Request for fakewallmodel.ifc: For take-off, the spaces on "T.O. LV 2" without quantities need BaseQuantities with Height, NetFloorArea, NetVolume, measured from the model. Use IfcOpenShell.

First a look at what the model holds.

```python
import ifcopenshell
import ifcopenshell.util.element
import ifcopenshell.util.unit

model = ifcopenshell.open("fakewallmodel.ifc")
print(model.schema)
for unit_type in ("LENGTHUNIT", "AREAUNIT", "VOLUMEUNIT"):
    print(unit_type, ifcopenshell.util.unit.calculate_unit_scale(model, unit_type))
storey = next(s for s in model.by_type("IfcBuildingStorey") if s.Name == "T.O. LV 2")
spaces = [e for e in ifcopenshell.util.element.get_decomposition(storey) if e.is_a("IfcSpace")]
for e in sorted(spaces, key=lambda e: e.id()):
    print(e.id(), e.is_a(), e.Name, list(ifcopenshell.util.element.get_psets(e, qtos_only=True)), sep=" | ")
```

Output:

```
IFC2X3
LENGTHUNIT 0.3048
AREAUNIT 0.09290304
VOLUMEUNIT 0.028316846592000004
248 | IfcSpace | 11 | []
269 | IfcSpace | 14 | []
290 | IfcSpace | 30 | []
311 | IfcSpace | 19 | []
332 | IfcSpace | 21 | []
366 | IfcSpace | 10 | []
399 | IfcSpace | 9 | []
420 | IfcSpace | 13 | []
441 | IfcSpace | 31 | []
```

```python
import ifcopenshell
import ifcopenshell.api.pset
import ifcopenshell.geom
import ifcopenshell.util.element
import ifcopenshell.util.shape
import ifcopenshell.util.unit

model = ifcopenshell.open("fakewallmodel.ifc")
unit_scale = ifcopenshell.util.unit.calculate_unit_scale(model)
area_scale = ifcopenshell.util.unit.calculate_unit_scale(model, "AREAUNIT")
volume_scale = ifcopenshell.util.unit.calculate_unit_scale(model, "VOLUMEUNIT")
settings = ifcopenshell.geom.settings()

storey = next(s for s in model.by_type("IfcBuildingStorey") if s.Name == "T.O. LV 2")
spaces = [e for e in ifcopenshell.util.element.get_decomposition(storey) if e.is_a("IfcSpace")]

for e in sorted(spaces, key=lambda e: e.id()):
    if ifcopenshell.util.element.get_psets(e, qtos_only=True, should_inherit=False):
        continue
    # Geometry comes back in metres, in the element's own axes.
    shape = ifcopenshell.geom.create_shape(settings, e)
    values = {
        "Height": ifcopenshell.util.shape.get_z(shape.geometry) / unit_scale,
        "NetFloorArea": ifcopenshell.util.shape.get_footprint_area(shape.geometry) / area_scale,
        "NetVolume": ifcopenshell.util.shape.get_volume(shape.geometry) / volume_scale,
    }
    qto = ifcopenshell.api.pset.add_qto(model, product=e, name="BaseQuantities")
    ifcopenshell.api.pset.edit_qto(model, qto=qto, properties=values)
    print(e.id(), {k: round(v, 3) for k, v in values.items()})

model.write("fakewallmodel-out.ifc")
```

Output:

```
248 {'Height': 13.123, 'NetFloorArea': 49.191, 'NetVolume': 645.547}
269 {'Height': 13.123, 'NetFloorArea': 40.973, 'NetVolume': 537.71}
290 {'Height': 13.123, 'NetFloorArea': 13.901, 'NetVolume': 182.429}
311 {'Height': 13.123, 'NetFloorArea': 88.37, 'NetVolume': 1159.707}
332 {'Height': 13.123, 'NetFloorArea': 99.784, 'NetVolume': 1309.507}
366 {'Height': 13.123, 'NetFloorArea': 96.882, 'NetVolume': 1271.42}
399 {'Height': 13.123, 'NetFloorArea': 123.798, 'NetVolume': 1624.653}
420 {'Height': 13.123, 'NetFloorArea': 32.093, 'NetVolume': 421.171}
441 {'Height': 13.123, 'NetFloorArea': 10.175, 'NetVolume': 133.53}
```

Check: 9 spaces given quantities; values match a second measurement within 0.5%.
